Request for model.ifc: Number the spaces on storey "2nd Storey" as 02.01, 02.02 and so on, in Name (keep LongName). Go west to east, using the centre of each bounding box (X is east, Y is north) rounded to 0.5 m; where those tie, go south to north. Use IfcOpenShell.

First a look at what the model holds.

```python
import ifcopenshell
import ifcopenshell.util.element
import ifcopenshell.util.placement

model = ifcopenshell.open("model.ifc")
print(model.schema)
storey = next(s for s in model.by_type("IfcBuildingStorey") if s.Name == "2nd Storey")
spaces = [e for e in ifcopenshell.util.element.get_decomposition(storey) if e.is_a("IfcSpace")]
for e in sorted(spaces, key=lambda e: e.id()):
    origin = ifcopenshell.util.placement.get_local_placement(e.ObjectPlacement)[:3, 3]
    print(e.id(), e.Name, e.LongName, origin.round(2) + 0.0, sep=" | ")
```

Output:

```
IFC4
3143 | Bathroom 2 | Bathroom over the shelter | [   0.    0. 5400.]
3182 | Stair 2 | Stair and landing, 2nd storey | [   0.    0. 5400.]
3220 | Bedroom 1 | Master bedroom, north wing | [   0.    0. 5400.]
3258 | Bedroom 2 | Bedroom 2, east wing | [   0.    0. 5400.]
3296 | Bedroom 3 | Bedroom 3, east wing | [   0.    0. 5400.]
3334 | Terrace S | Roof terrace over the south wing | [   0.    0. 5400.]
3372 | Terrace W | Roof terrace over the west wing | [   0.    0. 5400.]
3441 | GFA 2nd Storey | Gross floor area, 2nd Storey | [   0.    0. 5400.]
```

```python
import ifcopenshell
import ifcopenshell.geom
import ifcopenshell.util.element
import ifcopenshell.util.shape

model = ifcopenshell.open("model.ifc")
settings = ifcopenshell.geom.settings()
settings.set("use-world-coords", True)


def centre(element):
    shape = ifcopenshell.geom.create_shape(settings, element)
    return ifcopenshell.util.shape.get_bbox_centroid(shape.geometry)


storey = next(s for s in model.by_type("IfcBuildingStorey") if s.Name == "2nd Storey")
spaces = [e for e in ifcopenshell.util.element.get_decomposition(storey) if e.is_a("IfcSpace")]

# Insertion points can sit at a corner or the storey origin, so sort by the geometry (in metres).
centres = {e: centre(e) for e in spaces}
spaces.sort(key=lambda e: (round(centres[e][0] / 0.5), centres[e][1]))

for i, e in enumerate(spaces, start=1):
    number = f"02.{i:02d}"
    e.Name = number
    print(e.id(), number)

model.write("model_updated.ifc")
```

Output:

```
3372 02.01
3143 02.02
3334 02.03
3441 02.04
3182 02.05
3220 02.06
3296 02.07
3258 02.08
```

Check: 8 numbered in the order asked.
